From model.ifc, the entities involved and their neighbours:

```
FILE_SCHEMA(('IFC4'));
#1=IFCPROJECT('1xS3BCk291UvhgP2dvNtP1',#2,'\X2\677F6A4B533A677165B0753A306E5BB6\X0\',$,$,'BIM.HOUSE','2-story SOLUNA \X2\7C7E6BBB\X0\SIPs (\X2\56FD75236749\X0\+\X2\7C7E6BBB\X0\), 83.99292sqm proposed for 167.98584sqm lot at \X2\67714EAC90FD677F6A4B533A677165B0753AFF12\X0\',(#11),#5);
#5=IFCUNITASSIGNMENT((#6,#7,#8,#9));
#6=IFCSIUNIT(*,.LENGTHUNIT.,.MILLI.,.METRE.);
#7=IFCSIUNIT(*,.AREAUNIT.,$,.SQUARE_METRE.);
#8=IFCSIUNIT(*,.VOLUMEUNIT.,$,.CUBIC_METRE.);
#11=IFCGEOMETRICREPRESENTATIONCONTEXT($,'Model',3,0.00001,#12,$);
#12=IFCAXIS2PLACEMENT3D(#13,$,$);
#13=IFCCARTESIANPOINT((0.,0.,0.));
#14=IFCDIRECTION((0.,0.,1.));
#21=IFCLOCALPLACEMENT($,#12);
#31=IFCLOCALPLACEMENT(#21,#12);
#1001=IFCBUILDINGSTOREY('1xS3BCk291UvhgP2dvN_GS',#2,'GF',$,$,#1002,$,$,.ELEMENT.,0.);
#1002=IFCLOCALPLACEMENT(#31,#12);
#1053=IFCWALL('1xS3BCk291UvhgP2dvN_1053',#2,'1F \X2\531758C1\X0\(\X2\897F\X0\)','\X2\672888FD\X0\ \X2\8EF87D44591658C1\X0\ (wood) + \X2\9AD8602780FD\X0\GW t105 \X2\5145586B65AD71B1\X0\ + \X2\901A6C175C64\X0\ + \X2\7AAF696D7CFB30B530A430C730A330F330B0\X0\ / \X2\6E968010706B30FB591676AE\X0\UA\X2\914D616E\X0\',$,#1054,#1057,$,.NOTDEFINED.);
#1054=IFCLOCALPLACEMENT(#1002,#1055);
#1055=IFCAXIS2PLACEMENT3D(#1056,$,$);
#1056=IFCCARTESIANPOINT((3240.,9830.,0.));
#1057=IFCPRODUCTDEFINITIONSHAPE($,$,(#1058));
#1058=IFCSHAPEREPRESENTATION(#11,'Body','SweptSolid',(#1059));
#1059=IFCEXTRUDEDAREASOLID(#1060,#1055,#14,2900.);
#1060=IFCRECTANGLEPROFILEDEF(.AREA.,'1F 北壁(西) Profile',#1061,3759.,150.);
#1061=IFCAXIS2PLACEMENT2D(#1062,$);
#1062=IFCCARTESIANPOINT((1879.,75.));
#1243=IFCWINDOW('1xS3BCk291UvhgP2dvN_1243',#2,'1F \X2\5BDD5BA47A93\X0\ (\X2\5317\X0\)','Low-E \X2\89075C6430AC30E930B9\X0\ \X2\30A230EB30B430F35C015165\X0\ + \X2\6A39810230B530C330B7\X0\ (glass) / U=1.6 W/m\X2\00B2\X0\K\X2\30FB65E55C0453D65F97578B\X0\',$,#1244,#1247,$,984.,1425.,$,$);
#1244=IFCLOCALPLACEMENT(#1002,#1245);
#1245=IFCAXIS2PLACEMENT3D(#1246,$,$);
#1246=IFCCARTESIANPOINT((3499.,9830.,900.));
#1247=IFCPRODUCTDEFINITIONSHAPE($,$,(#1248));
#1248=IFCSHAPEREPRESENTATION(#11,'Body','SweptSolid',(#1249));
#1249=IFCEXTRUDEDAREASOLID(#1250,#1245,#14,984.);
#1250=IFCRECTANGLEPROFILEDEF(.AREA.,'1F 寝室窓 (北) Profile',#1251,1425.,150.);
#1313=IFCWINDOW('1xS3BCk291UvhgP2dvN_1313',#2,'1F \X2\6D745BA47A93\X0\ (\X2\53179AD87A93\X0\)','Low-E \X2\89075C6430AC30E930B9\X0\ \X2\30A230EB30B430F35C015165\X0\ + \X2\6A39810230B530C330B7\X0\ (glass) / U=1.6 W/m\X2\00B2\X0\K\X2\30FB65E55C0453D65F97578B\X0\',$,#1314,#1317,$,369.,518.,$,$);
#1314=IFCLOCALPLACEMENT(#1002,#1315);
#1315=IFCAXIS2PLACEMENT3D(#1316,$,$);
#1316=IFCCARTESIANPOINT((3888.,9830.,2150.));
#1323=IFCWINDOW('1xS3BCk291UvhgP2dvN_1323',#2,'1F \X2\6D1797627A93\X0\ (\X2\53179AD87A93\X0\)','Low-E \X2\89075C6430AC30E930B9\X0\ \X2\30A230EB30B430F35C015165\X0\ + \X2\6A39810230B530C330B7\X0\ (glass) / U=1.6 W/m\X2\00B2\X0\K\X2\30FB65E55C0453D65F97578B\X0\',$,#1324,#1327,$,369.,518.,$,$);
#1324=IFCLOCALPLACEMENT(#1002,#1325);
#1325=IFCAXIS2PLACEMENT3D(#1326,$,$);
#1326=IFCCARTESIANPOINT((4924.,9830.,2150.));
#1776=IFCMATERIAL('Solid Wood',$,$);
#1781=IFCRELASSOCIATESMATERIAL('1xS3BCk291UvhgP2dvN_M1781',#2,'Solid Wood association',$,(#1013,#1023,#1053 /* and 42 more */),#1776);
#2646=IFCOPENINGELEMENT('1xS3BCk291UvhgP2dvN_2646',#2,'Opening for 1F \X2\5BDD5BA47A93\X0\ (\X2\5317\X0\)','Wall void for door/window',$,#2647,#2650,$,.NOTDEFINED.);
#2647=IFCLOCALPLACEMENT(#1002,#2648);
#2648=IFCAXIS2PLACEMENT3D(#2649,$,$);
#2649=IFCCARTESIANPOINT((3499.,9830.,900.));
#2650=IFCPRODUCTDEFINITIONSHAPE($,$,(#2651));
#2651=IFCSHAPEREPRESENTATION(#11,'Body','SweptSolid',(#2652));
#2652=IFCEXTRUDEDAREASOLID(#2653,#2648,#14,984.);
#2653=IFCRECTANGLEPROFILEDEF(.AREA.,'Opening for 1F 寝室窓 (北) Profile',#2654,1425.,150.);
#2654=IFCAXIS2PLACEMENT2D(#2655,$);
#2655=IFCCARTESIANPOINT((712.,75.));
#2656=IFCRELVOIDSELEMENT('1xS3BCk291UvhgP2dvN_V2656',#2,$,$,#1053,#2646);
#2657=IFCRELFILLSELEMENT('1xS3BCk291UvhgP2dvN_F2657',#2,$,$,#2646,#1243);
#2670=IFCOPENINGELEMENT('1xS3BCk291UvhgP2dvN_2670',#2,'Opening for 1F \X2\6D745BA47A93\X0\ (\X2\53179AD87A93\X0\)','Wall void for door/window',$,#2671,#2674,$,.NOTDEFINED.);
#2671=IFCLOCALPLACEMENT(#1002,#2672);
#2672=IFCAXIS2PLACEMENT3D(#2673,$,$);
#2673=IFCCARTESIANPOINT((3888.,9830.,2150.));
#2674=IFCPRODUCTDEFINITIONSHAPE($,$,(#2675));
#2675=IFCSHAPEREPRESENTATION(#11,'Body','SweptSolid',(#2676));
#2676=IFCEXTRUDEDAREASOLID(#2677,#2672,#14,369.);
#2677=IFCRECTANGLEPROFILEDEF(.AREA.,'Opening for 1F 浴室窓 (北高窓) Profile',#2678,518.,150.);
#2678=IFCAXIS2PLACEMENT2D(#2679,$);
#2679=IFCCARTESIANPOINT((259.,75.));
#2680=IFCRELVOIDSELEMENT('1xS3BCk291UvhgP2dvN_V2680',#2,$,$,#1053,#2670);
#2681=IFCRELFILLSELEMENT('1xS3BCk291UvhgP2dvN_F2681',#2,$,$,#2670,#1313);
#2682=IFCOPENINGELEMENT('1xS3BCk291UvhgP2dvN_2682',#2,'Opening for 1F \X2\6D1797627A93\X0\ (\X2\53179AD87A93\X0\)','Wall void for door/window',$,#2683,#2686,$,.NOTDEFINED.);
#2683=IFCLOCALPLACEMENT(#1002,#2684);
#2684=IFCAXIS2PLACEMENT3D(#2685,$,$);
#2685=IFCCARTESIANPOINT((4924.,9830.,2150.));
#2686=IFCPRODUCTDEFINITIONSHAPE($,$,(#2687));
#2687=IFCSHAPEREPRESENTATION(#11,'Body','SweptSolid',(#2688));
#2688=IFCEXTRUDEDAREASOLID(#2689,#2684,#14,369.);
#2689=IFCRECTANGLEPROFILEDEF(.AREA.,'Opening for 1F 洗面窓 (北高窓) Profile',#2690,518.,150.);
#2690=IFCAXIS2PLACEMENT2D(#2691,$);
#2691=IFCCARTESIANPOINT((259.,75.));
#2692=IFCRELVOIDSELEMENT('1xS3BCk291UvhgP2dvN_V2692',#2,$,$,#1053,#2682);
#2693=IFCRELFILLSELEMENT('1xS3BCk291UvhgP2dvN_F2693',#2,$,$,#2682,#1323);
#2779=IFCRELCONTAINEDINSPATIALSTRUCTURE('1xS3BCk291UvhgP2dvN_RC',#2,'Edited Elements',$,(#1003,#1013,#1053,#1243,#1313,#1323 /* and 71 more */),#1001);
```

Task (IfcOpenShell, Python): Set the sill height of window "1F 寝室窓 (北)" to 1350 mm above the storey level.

```python
import numpy as np
import ifcopenshell
import ifcopenshell.api.geometry
import ifcopenshell.geom
import ifcopenshell.util.element
import ifcopenshell.util.placement
import ifcopenshell.util.shape
import ifcopenshell.util.unit

model = ifcopenshell.open("model.ifc")
unit_scale = ifcopenshell.util.unit.calculate_unit_scale(model)

window = model.by_id(1243)
opening = window.FillsVoids[0].RelatingOpeningElement
storey = ifcopenshell.util.element.get_container(window, ifc_class="IfcBuildingStorey")
level = ifcopenshell.util.placement.get_local_placement(storey.ObjectPlacement)[2, 3]

# The opening's origin need not be at the sill, so measure its lowest point.
shape = ifcopenshell.geom.create_shape(ifcopenshell.geom.settings(), opening)
bottom = ifcopenshell.util.shape.get_shape_bottom_elevation(shape, shape.geometry) / unit_scale
dz = level + 1.35 / unit_scale - bottom

shift = np.array([0.0, 0.0, dz])
# The window is not placed relative to its opening, so move both.
for product in (opening, window):
    matrix = ifcopenshell.util.placement.get_local_placement(product.ObjectPlacement)
    matrix[:3, 3] += shift
    ifcopenshell.api.geometry.edit_object_placement(model, product=product, matrix=matrix, is_si=False)

print(f"moved by {dz * unit_scale:+.3f} m")

model.write("model_updated.ifc")
```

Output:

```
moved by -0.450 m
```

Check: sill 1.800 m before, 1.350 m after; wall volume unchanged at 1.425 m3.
